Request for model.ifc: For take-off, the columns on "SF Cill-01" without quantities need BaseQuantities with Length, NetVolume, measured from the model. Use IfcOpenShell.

First a look at what the model holds.

```python
import ifcopenshell
import ifcopenshell.util.element
import ifcopenshell.util.unit

model = ifcopenshell.open("model.ifc")
print(model.schema)
for unit_type in ("LENGTHUNIT", "AREAUNIT", "VOLUMEUNIT"):
    print(unit_type, ifcopenshell.util.unit.calculate_unit_scale(model, unit_type))
storey = next(s for s in model.by_type("IfcBuildingStorey") if s.Name == "SF Cill-01")
columns = [e for e in ifcopenshell.util.element.get_decomposition(storey) if e.is_a("IfcColumn")]
for e in sorted(columns, key=lambda e: e.id()):
    print(e.id(), e.is_a(), e.Name, list(ifcopenshell.util.element.get_psets(e, qtos_only=True)), sep=" | ")
```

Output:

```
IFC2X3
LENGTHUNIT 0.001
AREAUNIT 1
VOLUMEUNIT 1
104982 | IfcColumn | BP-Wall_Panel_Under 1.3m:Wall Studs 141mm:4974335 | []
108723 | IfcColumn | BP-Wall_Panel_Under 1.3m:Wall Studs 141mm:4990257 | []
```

```python
import ifcopenshell
import ifcopenshell.api.pset
import ifcopenshell.geom
import ifcopenshell.util.element
import ifcopenshell.util.shape
import ifcopenshell.util.unit

model = ifcopenshell.open("model.ifc")
unit_scale = ifcopenshell.util.unit.calculate_unit_scale(model)
volume_scale = ifcopenshell.util.unit.calculate_unit_scale(model, "VOLUMEUNIT")
settings = ifcopenshell.geom.settings()

storey = next(s for s in model.by_type("IfcBuildingStorey") if s.Name == "SF Cill-01")
columns = [e for e in ifcopenshell.util.element.get_decomposition(storey) if e.is_a("IfcColumn")]

for e in sorted(columns, key=lambda e: e.id()):
    if ifcopenshell.util.element.get_psets(e, qtos_only=True, should_inherit=False):
        continue
    # Geometry comes back in metres, in the element's own axes.
    shape = ifcopenshell.geom.create_shape(settings, e)
    values = {
        "Length": ifcopenshell.util.shape.get_z(shape.geometry) / unit_scale,
        "NetVolume": ifcopenshell.util.shape.get_volume(shape.geometry) / volume_scale,
    }
    qto = ifcopenshell.api.pset.add_qto(model, product=e, name="BaseQuantities")
    ifcopenshell.api.pset.edit_qto(model, qto=qto, properties=values)
    print(e.id(), {k: round(v, 3) for k, v in values.items()})

model.write("model-out.ifc")
```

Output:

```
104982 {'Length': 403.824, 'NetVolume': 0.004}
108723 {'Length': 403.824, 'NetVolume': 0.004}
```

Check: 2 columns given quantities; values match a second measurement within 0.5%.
